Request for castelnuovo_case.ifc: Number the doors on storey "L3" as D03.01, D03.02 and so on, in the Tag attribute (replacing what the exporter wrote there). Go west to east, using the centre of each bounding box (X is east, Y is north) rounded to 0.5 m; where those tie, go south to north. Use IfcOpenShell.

First a look at what the model holds.

```python
import ifcopenshell
import ifcopenshell.util.element
import ifcopenshell.util.placement

model = ifcopenshell.open("castelnuovo_case.ifc")
print(model.schema)
storey = next(s for s in model.by_type("IfcBuildingStorey") if s.Name == "L3")
doors = [e for e in ifcopenshell.util.element.get_decomposition(storey) if e.is_a("IfcDoor")]
for e in sorted(doors, key=lambda e: e.id()):
    origin = ifcopenshell.util.placement.get_local_placement(e.ObjectPlacement)[:3, 3]
    print(e.id(), e.Tag, e.Name, origin.round(2) + 0.0, sep=" | ")
```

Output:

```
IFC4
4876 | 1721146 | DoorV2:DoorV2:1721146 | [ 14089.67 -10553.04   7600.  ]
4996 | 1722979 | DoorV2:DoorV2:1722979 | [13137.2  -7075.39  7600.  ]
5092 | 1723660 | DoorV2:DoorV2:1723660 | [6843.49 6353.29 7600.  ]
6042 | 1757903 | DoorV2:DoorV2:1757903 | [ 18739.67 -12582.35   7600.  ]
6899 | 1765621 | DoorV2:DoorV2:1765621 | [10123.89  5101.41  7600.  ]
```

```python
import ifcopenshell
import ifcopenshell.geom
import ifcopenshell.util.element
import ifcopenshell.util.shape

model = ifcopenshell.open("castelnuovo_case.ifc")
settings = ifcopenshell.geom.settings()
settings.set("use-world-coords", True)


def centre(element):
    shape = ifcopenshell.geom.create_shape(settings, element)
    return ifcopenshell.util.shape.get_bbox_centroid(shape.geometry)


storey = next(s for s in model.by_type("IfcBuildingStorey") if s.Name == "L3")
doors = [e for e in ifcopenshell.util.element.get_decomposition(storey) if e.is_a("IfcDoor")]

# Insertion points can sit at a corner or the storey origin, so sort by the geometry (in metres).
centres = {e: centre(e) for e in doors}
doors.sort(key=lambda e: (round(centres[e][0] / 0.5), centres[e][1]))

for i, e in enumerate(doors, start=1):
    number = f"D03.{i:02d}"
    e.Tag = number
    print(e.id(), number)

model.write("castelnuovo_case_edited.ifc")
```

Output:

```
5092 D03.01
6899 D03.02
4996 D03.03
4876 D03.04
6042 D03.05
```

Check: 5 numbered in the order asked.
